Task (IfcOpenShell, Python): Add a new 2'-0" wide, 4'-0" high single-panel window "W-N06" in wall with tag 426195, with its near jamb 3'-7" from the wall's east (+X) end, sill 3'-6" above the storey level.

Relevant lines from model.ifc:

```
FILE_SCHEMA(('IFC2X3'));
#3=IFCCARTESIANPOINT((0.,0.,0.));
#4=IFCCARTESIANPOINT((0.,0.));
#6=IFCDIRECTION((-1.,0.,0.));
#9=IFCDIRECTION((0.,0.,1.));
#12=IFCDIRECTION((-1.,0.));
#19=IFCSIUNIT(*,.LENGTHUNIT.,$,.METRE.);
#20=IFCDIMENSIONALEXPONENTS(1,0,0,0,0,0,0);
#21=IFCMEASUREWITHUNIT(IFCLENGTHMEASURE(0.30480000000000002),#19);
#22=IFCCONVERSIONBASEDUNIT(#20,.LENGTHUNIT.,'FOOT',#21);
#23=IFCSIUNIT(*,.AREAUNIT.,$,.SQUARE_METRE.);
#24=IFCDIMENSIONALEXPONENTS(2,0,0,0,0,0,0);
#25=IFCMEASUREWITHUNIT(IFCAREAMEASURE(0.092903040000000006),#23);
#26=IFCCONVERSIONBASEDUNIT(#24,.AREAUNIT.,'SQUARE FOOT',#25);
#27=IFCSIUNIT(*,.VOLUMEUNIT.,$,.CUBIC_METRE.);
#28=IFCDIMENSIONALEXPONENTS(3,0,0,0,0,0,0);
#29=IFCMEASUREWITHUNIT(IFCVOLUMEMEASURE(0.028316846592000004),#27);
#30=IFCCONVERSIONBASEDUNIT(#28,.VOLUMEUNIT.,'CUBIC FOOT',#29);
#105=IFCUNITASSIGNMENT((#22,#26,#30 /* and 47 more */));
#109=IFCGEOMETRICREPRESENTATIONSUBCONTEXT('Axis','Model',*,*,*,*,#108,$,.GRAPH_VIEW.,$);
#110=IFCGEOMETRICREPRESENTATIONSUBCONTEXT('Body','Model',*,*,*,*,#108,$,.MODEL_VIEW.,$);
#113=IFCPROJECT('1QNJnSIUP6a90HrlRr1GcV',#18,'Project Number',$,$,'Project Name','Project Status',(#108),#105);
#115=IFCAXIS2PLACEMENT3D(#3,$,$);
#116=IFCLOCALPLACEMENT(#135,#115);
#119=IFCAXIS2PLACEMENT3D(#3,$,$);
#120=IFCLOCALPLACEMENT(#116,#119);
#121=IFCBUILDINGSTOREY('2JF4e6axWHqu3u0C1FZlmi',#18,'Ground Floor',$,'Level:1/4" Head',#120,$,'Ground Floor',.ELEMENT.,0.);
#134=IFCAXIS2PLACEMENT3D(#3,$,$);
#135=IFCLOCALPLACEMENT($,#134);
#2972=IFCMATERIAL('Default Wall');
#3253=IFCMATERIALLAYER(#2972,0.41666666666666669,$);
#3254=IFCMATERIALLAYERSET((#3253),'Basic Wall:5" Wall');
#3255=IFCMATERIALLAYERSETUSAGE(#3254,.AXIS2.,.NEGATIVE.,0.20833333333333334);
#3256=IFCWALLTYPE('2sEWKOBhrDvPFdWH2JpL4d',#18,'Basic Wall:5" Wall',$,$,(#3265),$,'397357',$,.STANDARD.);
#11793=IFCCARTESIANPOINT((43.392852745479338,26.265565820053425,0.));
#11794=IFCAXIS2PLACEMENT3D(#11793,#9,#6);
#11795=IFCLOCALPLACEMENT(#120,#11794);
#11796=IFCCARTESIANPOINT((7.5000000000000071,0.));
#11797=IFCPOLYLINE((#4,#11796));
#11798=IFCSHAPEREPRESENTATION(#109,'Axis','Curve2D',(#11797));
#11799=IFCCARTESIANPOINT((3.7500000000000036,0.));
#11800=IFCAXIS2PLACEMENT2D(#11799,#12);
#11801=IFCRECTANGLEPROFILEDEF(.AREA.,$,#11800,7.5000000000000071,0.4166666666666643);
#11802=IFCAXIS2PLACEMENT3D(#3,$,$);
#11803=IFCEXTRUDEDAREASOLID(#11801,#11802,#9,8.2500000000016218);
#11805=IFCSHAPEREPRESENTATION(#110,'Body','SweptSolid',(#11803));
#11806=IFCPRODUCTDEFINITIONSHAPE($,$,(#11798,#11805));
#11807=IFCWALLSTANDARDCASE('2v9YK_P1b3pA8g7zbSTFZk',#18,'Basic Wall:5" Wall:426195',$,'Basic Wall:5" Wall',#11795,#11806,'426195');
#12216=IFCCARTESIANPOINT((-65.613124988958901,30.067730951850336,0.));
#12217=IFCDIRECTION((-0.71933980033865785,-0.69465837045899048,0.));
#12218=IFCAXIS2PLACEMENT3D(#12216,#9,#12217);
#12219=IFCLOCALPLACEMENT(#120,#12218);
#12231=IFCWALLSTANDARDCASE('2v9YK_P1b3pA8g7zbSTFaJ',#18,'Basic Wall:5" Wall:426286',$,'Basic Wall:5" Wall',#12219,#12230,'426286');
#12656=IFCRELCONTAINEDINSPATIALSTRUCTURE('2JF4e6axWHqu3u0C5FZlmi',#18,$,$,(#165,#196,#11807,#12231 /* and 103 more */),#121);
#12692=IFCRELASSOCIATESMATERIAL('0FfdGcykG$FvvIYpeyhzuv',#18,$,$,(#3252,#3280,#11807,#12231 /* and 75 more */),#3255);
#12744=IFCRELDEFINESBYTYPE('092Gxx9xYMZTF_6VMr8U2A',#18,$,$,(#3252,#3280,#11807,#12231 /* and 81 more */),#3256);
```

```python
import numpy as np
import ifcopenshell
import ifcopenshell.api.feature
import ifcopenshell.api.geometry
import ifcopenshell.api.root
import ifcopenshell.api.spatial
import ifcopenshell.api.type
import ifcopenshell.geom
import ifcopenshell.util.element
import ifcopenshell.util.placement
import ifcopenshell.util.representation
import ifcopenshell.util.shape
import ifcopenshell.util.unit

model = ifcopenshell.open("model.ifc")
unit_scale = ifcopenshell.util.unit.calculate_unit_scale(model)
settings = ifcopenshell.geom.settings()


def volume(element):
    """Net volume in cubic metres, openings subtracted."""
    shape = ifcopenshell.geom.create_shape(settings, element)
    return ifcopenshell.util.shape.get_volume(shape.geometry)


wall = model.by_id(11807)
storey = ifcopenshell.util.element.get_container(wall, ifc_class="IfcBuildingStorey")
context = ifcopenshell.util.representation.get_context(model, "Model", "Body", "MODEL_VIEW")
before = volume(wall)

width, height, from_end, sill = 0.6096, 1.2192, 1.0922, 1.0668  # metres

# The wall runs along its own X axis, and the end named is its -X end.
wall_shape = ifcopenshell.geom.create_shape(settings, wall)
x, y, z = ifcopenshell.util.shape.get_vertices(wall_shape.geometry).T
start = x.min() + from_end
face, thickness = float(y.min()), float(y.max() - y.min())
wall_matrix = ifcopenshell.util.placement.get_local_placement(wall.ObjectPlacement)
level = ifcopenshell.util.placement.get_local_placement(storey.ObjectPlacement)[2, 3]


def in_wall(x, y):
    """Placement at x, y metres in the wall's axes, at sill height."""
    matrix = wall_matrix.copy()
    matrix[:, 3] = wall_matrix @ np.array([x / unit_scale, y / unit_scale, 0.0, 1.0])
    matrix[2, 3] = level + sill / unit_scale
    return matrix


# Opening: a box that overshoots both wall faces by 50 mm.
opening = ifcopenshell.api.root.create_entity(model, ifc_class="IfcOpeningElement")
box = ifcopenshell.api.geometry.add_wall_representation(
    model, context=context, length=width, height=height, thickness=thickness + 0.1
)
ifcopenshell.api.geometry.assign_representation(model, product=opening, representation=box)
ifcopenshell.api.geometry.edit_object_placement(model, product=opening, matrix=in_wall(start, face - 0.05), is_si=False)
ifcopenshell.api.feature.add_feature(model, feature=opening, element=wall)

window = ifcopenshell.api.root.create_entity(model, ifc_class="IfcWindow", name="W-N06")
window.OverallWidth, window.OverallHeight = width / unit_scale, height / unit_scale
body = ifcopenshell.api.geometry.add_window_representation(
    model,
    context=context,
    overall_width=window.OverallWidth,
    overall_height=window.OverallHeight,
    partition_type="SINGLE_PANEL",
)
ifcopenshell.api.geometry.assign_representation(model, product=window, representation=body)
ifcopenshell.api.spatial.assign_container(model, products=[window], relating_structure=storey)
fills = ifcopenshell.api.feature.add_filling(model, opening=opening, element=window)
fills.OwnerHistory = window.OwnerHistory  # required in IFC2X3

# IFC2X3 keeps the operation on the window style.
style = ifcopenshell.api.root.create_entity(model, ifc_class="IfcWindowStyle", name="W-N06")
style.OperationType, style.ConstructionType = "SINGLE_PANEL", "NOTDEFINED"
style.ParameterTakesPrecedence = style.Sizeable = False
ifcopenshell.api.type.assign_type(model, related_objects=[window], relating_type=style)

# Centre the window in the wall's thickness.
ifcopenshell.api.geometry.edit_object_placement(model, product=window, matrix=in_wall(start, face), is_si=False)
window_shape = ifcopenshell.geom.create_shape(settings, window)
depth = ifcopenshell.util.shape.get_vertices(window_shape.geometry)[:, 1]
offset = face + thickness / 2 - (depth.min() + depth.max()) / 2
ifcopenshell.api.geometry.edit_object_placement(model, product=window, matrix=in_wall(start, offset), is_si=False)

after = volume(wall)

print(f"wall volume {before:.3f} -> {after:.3f} m3")

model.write("model-out.ifc")
```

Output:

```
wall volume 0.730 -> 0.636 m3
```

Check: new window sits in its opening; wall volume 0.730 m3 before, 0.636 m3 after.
